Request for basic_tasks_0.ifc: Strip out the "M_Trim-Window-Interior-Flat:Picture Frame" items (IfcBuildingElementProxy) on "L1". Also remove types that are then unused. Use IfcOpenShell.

First a look at what the model holds.

```python
import ifcopenshell
import ifcopenshell.util.element

model = ifcopenshell.open("basic_tasks_0.ifc")
print(model.schema)
storey = next(s for s in model.by_type("IfcBuildingStorey") if s.Name == "L1")
proxies = [e for e in ifcopenshell.util.element.get_decomposition(storey) if e.is_a("IfcBuildingElementProxy")]
seen = {}
for e in proxies:
    element_type = ifcopenshell.util.element.get_type(e)
    name = element_type.Name if element_type not in (None, e) else None
    seen[name] = seen.get(name, 0) + 1
for name, count in sorted(seen.items(), key=str):
    print(count, "x", name)
```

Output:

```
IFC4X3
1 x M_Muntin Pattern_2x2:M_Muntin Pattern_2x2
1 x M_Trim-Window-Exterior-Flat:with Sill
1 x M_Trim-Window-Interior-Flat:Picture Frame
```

```python
import ifcopenshell
import ifcopenshell.api.root
import ifcopenshell.util.element

model = ifcopenshell.open("basic_tasks_0.ifc")

storey = next(s for s in model.by_type("IfcBuildingStorey") if s.Name == "L1")
proxies = [e for e in ifcopenshell.util.element.get_decomposition(storey) if e.is_a("IfcBuildingElementProxy")]
targets = [e for e in proxies if (t := ifcopenshell.util.element.get_type(e)) not in (None, e) and t.Name == "M_Trim-Window-Interior-Flat:Picture Frame"]
types = {ifcopenshell.util.element.get_type(e) for e in targets} - {None, *targets}

for e in targets:
    ifcopenshell.api.root.remove_product(model, product=e)
print(len(targets), "removed")

unused = [t for t in types if not ifcopenshell.util.element.get_types(t)]
for t in unused:
    ifcopenshell.api.root.remove_product(model, product=t)
print(len(unused), "unused types removed")

model.write("basic_tasks_0-out.ifc")
```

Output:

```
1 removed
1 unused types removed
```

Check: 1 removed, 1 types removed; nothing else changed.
